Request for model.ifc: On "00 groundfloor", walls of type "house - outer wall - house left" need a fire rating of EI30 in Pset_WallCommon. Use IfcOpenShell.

First a look at what the model holds.

```python
import ifcopenshell
import ifcopenshell.util.element

model = ifcopenshell.open("model.ifc")
print(model.schema)
storey = next(s for s in model.by_type("IfcBuildingStorey") if s.Name == "00 groundfloor")
walls = [e for e in ifcopenshell.util.element.get_decomposition(storey) if e.is_a("IfcWall")]
seen = {}
for e in walls:
    element_type = ifcopenshell.util.element.get_type(e)
    key = (element_type.Name if element_type != e and element_type else None, ifcopenshell.util.element.get_pset(e, "Pset_WallCommon", "FireRating"))
    seen[key] = seen.get(key, 0) + 1
for (name, value), count in sorted(seen.items(), key=str):
    print(count, "x", name, "|", value)
```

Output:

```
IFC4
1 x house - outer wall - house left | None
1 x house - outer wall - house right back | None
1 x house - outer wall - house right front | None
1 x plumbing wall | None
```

```python
import ifcopenshell
import ifcopenshell.api.pset
import ifcopenshell.util.element

model = ifcopenshell.open("model.ifc")

storey = next(s for s in model.by_type("IfcBuildingStorey") if s.Name == "00 groundfloor")
walls = [e for e in ifcopenshell.util.element.get_decomposition(storey) if e.is_a("IfcWall")]

count = 0
for e in walls:
    element_type = ifcopenshell.util.element.get_type(e)
    if element_type in (None, e) or element_type.Name != "house - outer wall - house left":
        continue
    # add_pset returns the element's existing set when there is one.
    pset = ifcopenshell.api.pset.add_pset(model, product=e, name="Pset_WallCommon")
    ifcopenshell.api.pset.edit_pset(model, pset=pset, properties={"FireRating": "EI30"})
    count += 1

print(count, "walls updated")

model.write("model_rev.ifc")
```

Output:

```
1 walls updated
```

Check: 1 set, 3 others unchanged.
